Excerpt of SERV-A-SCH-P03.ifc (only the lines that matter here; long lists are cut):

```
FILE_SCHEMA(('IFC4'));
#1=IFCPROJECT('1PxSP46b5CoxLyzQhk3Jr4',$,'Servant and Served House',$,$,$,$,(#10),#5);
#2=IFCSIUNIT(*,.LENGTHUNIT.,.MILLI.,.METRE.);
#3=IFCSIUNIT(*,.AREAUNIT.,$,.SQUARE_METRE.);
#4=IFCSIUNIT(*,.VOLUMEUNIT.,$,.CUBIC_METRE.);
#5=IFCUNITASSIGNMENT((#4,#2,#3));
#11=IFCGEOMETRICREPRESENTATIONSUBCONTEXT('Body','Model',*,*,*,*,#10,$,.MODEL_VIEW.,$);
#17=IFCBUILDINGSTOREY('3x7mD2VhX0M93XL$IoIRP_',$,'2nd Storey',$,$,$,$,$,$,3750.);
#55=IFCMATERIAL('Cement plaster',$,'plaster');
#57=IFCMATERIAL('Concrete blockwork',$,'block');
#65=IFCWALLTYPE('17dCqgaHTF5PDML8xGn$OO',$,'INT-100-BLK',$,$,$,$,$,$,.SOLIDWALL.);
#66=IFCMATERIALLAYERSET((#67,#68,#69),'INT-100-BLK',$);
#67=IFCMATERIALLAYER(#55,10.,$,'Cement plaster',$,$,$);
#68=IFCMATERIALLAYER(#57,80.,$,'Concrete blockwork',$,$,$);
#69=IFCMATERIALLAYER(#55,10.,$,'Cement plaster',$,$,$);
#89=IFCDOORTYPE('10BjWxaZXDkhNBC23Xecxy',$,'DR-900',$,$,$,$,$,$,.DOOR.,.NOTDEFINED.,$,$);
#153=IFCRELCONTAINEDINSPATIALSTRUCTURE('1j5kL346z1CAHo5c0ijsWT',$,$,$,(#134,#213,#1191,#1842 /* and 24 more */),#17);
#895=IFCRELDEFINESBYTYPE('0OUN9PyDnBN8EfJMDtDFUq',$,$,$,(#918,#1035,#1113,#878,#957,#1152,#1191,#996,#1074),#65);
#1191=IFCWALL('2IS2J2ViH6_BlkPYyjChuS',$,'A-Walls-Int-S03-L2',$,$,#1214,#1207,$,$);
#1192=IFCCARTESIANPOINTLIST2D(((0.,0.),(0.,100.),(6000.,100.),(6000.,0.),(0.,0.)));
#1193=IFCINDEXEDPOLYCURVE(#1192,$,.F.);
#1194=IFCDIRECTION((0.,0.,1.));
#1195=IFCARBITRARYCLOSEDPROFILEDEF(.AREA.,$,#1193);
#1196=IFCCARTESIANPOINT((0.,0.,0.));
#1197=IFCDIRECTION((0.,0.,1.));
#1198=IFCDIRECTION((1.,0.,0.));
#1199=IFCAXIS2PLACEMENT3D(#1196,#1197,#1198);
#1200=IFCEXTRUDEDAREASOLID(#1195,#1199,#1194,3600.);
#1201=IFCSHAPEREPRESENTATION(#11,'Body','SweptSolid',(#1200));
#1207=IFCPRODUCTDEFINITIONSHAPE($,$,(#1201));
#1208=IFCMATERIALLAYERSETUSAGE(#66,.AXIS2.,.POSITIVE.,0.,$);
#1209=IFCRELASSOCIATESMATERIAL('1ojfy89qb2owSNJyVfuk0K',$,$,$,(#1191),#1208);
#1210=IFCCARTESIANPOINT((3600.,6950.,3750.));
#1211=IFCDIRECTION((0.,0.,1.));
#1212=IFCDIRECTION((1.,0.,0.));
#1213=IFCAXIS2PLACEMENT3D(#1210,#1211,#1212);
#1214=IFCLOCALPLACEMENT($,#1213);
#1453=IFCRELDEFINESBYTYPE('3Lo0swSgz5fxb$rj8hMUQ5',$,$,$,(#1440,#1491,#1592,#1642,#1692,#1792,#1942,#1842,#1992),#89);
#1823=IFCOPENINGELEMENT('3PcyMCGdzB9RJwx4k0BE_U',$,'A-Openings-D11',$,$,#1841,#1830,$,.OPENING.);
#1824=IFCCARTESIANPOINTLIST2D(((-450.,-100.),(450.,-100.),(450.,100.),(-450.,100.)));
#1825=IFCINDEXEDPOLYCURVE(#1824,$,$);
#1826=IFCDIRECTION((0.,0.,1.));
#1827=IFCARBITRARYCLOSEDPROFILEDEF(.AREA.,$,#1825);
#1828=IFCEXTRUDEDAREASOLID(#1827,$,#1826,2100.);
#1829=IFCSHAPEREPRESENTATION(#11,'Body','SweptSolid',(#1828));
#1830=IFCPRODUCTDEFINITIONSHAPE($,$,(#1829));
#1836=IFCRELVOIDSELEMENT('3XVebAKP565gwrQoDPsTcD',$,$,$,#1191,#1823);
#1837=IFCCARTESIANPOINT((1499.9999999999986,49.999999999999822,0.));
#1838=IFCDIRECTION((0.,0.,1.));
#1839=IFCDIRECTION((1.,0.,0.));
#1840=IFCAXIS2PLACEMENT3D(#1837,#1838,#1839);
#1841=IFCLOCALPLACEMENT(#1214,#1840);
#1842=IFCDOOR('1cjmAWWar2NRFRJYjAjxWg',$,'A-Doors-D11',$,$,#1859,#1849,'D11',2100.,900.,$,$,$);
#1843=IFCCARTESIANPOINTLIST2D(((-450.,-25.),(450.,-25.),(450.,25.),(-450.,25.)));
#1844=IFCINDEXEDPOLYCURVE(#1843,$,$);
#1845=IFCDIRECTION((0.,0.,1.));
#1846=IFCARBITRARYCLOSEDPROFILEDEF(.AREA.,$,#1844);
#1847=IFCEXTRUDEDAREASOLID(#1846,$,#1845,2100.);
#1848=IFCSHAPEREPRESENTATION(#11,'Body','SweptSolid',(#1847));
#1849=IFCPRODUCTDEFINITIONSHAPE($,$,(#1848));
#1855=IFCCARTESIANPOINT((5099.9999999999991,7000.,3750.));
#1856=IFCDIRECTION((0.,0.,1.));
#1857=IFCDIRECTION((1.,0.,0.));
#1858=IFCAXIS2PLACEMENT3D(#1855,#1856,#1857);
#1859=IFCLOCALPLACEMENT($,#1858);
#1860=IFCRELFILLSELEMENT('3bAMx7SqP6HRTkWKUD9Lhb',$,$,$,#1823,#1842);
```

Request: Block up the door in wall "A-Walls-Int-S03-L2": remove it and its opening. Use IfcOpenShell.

```python
import ifcopenshell
import ifcopenshell.api.feature
import ifcopenshell.api.root
import ifcopenshell.geom
import ifcopenshell.util.shape

model = ifcopenshell.open("SERV-A-SCH-P03.ifc")
settings = ifcopenshell.geom.settings()


def volume(element):
    """Net volume in cubic metres, openings subtracted."""
    shape = ifcopenshell.geom.create_shape(settings, element)
    return ifcopenshell.util.shape.get_volume(shape.geometry)


door = model.by_guid("1cjmAWWar2NRFRJYjAjxWg")
opening = door.FillsVoids[0].RelatingOpeningElement
wall = opening.VoidsElements[0].RelatingBuildingElement
before = volume(wall)

ifcopenshell.api.root.remove_product(model, product=door)
ifcopenshell.api.feature.remove_feature(model, feature=opening)

after = volume(wall)

print(f"wall volume {before:.3f} -> {after:.3f} m3")

model.write("SERV-A-SCH-P03-out.ifc")
```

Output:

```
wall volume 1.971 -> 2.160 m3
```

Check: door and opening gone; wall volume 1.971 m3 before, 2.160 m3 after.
